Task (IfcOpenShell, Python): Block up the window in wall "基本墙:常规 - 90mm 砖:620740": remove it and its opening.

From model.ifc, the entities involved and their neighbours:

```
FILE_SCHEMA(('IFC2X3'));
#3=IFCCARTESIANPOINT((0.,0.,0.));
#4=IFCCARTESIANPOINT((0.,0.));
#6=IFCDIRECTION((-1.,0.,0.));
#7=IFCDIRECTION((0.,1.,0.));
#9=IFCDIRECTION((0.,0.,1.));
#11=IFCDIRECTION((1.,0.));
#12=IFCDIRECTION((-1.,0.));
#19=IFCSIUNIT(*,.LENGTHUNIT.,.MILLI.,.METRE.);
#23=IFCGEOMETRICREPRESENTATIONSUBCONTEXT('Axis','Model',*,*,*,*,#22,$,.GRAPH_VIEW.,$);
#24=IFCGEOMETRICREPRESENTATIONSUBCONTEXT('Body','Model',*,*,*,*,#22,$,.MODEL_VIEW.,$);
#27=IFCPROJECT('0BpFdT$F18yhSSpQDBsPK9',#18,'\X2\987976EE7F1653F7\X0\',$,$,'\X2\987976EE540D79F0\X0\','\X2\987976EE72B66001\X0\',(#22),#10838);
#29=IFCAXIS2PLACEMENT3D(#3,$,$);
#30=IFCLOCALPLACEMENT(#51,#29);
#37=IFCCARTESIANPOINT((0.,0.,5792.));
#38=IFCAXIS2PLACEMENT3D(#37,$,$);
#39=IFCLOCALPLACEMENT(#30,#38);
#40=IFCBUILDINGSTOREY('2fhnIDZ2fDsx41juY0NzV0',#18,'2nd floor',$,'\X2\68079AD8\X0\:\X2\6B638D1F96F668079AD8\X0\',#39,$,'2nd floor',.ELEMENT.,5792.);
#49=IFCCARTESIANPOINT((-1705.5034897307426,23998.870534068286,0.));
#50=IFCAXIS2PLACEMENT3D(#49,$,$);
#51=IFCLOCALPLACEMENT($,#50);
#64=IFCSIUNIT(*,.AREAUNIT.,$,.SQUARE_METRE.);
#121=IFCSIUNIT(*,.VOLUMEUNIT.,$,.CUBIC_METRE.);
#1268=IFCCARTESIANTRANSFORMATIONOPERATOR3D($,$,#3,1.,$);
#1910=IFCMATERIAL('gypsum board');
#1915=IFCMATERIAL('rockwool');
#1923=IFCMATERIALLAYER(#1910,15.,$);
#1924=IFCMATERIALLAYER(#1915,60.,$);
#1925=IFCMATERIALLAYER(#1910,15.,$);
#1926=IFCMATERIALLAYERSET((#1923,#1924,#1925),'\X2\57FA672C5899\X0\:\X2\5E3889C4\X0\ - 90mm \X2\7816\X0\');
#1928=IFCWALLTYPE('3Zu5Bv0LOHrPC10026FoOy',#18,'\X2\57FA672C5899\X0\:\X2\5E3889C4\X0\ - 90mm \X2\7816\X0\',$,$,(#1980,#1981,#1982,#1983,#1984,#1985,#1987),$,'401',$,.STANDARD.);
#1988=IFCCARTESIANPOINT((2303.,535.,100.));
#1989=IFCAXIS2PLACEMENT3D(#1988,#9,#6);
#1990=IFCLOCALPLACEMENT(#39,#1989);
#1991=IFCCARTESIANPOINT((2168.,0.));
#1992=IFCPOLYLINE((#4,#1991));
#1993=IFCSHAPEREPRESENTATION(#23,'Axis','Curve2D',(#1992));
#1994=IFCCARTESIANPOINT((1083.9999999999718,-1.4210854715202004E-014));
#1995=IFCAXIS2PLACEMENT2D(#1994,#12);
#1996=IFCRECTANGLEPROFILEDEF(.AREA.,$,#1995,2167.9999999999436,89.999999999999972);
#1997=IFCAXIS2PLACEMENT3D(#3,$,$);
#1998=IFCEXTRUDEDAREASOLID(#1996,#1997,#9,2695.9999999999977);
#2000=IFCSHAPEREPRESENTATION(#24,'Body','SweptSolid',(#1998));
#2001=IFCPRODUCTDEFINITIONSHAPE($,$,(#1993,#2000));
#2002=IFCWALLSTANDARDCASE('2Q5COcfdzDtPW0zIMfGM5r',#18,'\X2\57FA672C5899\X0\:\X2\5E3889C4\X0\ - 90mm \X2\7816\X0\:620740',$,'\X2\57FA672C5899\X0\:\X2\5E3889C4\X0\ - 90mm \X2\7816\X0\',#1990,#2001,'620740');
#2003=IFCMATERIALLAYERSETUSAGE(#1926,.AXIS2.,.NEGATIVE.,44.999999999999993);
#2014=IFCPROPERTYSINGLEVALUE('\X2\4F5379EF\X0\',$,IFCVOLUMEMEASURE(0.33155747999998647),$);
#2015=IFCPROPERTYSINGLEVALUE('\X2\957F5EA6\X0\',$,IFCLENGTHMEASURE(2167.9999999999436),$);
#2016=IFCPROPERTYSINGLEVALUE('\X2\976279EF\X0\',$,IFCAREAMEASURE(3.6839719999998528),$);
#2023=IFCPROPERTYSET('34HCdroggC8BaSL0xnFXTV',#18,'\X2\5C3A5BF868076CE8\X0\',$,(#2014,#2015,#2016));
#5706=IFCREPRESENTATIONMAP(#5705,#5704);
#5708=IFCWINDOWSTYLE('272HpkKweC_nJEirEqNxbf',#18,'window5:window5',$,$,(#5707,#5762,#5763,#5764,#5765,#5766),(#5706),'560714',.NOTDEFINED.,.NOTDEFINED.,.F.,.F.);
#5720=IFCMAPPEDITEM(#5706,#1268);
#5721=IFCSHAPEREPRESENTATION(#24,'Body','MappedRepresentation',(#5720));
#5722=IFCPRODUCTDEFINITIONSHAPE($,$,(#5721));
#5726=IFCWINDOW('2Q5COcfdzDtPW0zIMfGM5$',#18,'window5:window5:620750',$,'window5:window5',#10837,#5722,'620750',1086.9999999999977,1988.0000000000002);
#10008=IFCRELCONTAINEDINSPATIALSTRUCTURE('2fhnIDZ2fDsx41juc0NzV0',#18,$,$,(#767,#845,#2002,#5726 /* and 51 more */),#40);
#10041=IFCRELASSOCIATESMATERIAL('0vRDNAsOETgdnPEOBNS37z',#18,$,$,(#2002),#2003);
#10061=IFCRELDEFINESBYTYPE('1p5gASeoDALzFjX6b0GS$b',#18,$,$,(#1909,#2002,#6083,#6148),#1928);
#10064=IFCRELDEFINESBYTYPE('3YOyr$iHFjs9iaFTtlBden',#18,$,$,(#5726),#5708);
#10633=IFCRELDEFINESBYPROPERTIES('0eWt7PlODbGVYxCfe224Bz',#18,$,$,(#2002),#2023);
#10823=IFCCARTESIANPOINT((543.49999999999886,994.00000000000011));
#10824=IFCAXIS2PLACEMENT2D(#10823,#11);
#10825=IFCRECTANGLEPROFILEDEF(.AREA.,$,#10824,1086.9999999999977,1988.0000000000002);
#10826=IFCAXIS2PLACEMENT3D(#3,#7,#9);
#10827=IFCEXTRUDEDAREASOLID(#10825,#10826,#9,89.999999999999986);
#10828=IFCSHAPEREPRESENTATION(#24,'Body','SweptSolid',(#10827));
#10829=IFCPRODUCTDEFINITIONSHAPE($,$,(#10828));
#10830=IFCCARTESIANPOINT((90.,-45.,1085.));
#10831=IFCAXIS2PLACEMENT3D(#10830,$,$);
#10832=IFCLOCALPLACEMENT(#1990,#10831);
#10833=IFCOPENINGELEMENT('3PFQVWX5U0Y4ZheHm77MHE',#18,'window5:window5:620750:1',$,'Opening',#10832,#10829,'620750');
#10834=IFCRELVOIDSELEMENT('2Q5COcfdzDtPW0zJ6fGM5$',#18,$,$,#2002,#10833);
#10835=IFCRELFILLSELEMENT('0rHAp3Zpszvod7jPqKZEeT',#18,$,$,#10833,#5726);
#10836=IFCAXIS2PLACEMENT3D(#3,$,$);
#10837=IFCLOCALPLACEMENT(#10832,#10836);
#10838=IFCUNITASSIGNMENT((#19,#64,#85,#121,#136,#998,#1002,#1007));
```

```python
import ifcopenshell
import ifcopenshell.api.feature
import ifcopenshell.api.pset
import ifcopenshell.api.root
import ifcopenshell.geom
import ifcopenshell.util.element
import ifcopenshell.util.shape
import ifcopenshell.util.unit

model = ifcopenshell.open("model.ifc")
area_scale = ifcopenshell.util.unit.calculate_unit_scale(model, "AREAUNIT")
volume_scale = ifcopenshell.util.unit.calculate_unit_scale(model, "VOLUMEUNIT")
settings = ifcopenshell.geom.settings()


def volume(element):
    """Net volume in cubic metres, openings subtracted."""
    shape = ifcopenshell.geom.create_shape(settings, element)
    return ifcopenshell.util.shape.get_volume(shape.geometry)


window = model.by_id(5726)
opening = window.FillsVoids[0].RelatingOpeningElement
wall = opening.VoidsElements[0].RelatingBuildingElement
before = volume(wall)

ifcopenshell.api.root.remove_product(model, product=window)
ifcopenshell.api.feature.remove_feature(model, feature=opening)

after = volume(wall)
thickness = 0.09  # wall thickness in metres

# Update the wall's stored quantities.
pset = model.by_id(ifcopenshell.util.element.get_pset(wall, "尺寸标注", should_inherit=False)["id"])
ifcopenshell.api.pset.edit_pset(model, pset=pset, properties={
    "体积": model.create_entity("IfcVolumeMeasure", after / volume_scale),
    "面积": model.create_entity("IfcAreaMeasure", after / thickness / area_scale),
})

print(f"wall volume {before:.3f} -> {after:.3f} m3")

model.write("model_v2.ifc")
```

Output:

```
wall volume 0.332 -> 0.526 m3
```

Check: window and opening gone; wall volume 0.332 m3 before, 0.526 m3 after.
